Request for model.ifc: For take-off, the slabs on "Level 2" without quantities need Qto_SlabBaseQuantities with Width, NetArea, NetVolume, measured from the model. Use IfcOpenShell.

First a look at what the model holds.

```python
import ifcopenshell
import ifcopenshell.util.element
import ifcopenshell.util.unit

model = ifcopenshell.open("model.ifc")
print(model.schema)
for unit_type in ("LENGTHUNIT", "AREAUNIT", "VOLUMEUNIT"):
    print(unit_type, ifcopenshell.util.unit.calculate_unit_scale(model, unit_type))
storey = next(s for s in model.by_type("IfcBuildingStorey") if s.Name == "Level 2")
slabs = [e for e in ifcopenshell.util.element.get_decomposition(storey) if e.is_a("IfcSlab")]
for e in sorted(slabs, key=lambda e: e.id()):
    print(e.id(), e.is_a(), e.Name, list(ifcopenshell.util.element.get_psets(e, qtos_only=True)), sep=" | ")
```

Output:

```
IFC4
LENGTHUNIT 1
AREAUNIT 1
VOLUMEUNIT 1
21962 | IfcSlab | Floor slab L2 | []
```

```python
import ifcopenshell
import ifcopenshell.api.pset
import ifcopenshell.geom
import ifcopenshell.util.element
import ifcopenshell.util.shape
import ifcopenshell.util.unit

model = ifcopenshell.open("model.ifc")
unit_scale = ifcopenshell.util.unit.calculate_unit_scale(model)
area_scale = ifcopenshell.util.unit.calculate_unit_scale(model, "AREAUNIT")
volume_scale = ifcopenshell.util.unit.calculate_unit_scale(model, "VOLUMEUNIT")
settings = ifcopenshell.geom.settings()

storey = next(s for s in model.by_type("IfcBuildingStorey") if s.Name == "Level 2")
slabs = [e for e in ifcopenshell.util.element.get_decomposition(storey) if e.is_a("IfcSlab")]

for e in sorted(slabs, key=lambda e: e.id()):
    if ifcopenshell.util.element.get_psets(e, qtos_only=True, should_inherit=False):
        continue
    # Geometry comes back in metres, in the element's own axes.
    shape = ifcopenshell.geom.create_shape(settings, e)
    values = {
        "Width": ifcopenshell.util.shape.get_z(shape.geometry) / unit_scale,
        "NetArea": ifcopenshell.util.shape.get_footprint_area(shape.geometry) / area_scale,
        "NetVolume": ifcopenshell.util.shape.get_volume(shape.geometry) / volume_scale,
    }
    qto = ifcopenshell.api.pset.add_qto(model, product=e, name="Qto_SlabBaseQuantities")
    ifcopenshell.api.pset.edit_qto(model, qto=qto, properties=values)
    print(e.id(), {k: round(v, 3) for k, v in values.items()})

model.write("model-out.ifc")
```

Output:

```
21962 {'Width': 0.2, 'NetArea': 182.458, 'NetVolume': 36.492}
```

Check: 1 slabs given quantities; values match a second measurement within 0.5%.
